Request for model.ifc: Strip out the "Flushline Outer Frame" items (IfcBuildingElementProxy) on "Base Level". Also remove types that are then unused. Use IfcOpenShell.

First a look at what the model holds.

```python
import ifcopenshell
import ifcopenshell.util.element

model = ifcopenshell.open("model.ifc")
print(model.schema)
storey = next(s for s in model.by_type("IfcBuildingStorey") if s.Name == "Base Level")
proxies = [e for e in ifcopenshell.util.element.get_decomposition(storey) if e.is_a("IfcBuildingElementProxy")]
seen = {}
for e in proxies:
    element_type = ifcopenshell.util.element.get_type(e)
    name = element_type.Name if element_type not in (None, e) else None
    seen[name] = seen.get(name, 0) + 1
for name, count in sorted(seen.items(), key=str):
    print(count, "x", name)
```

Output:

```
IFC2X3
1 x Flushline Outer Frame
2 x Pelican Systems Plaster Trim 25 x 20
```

```python
import ifcopenshell
import ifcopenshell.api.root
import ifcopenshell.util.element

model = ifcopenshell.open("model.ifc")

storey = next(s for s in model.by_type("IfcBuildingStorey") if s.Name == "Base Level")
proxies = [e for e in ifcopenshell.util.element.get_decomposition(storey) if e.is_a("IfcBuildingElementProxy")]
targets = [e for e in proxies if (t := ifcopenshell.util.element.get_type(e)) not in (None, e) and t.Name == "Flushline Outer Frame"]
types = {ifcopenshell.util.element.get_type(e) for e in targets} - {None, *targets}

for e in targets:
    ifcopenshell.api.root.remove_product(model, product=e)
print(len(targets), "removed")

unused = [t for t in types if not ifcopenshell.util.element.get_types(t)]
for t in unused:
    ifcopenshell.api.root.remove_product(model, product=t)
print(len(unused), "unused types removed")

model.write("model_updated.ifc")
```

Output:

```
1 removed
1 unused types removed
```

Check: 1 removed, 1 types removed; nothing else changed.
